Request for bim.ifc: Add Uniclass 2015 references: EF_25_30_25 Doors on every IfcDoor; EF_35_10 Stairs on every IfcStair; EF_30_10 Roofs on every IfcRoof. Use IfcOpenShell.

First a look at what the model holds.

```python
import ifcopenshell

model = ifcopenshell.open("bim.ifc")
print(model.schema)
print("classifications:", [c.Name for c in model.by_type("IfcClassification")])
for ifc_class in ("IfcDoor", "IfcRoof", "IfcStair", "IfcWall", "IfcWindow"):
    print(ifc_class, len(model.by_type(ifc_class)))
```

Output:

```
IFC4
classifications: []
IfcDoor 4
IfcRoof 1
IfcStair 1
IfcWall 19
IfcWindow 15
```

```python
import ifcopenshell
import ifcopenshell.api.classification

model = ifcopenshell.open("bim.ifc")

system = ifcopenshell.api.classification.add_classification(model, classification="Uniclass 2015")

codes = {
    "IfcDoor": ("EF_25_30_25", "Doors"),
    "IfcStair": ("EF_35_10", "Stairs"),
    "IfcRoof": ("EF_30_10", "Roofs"),
}
for ifc_class, (code, name) in codes.items():
    products = model.by_type(ifc_class)
    ifcopenshell.api.classification.add_reference(
        model, products=products, classification=system, identification=code, name=name
    )
    print(code, len(products))

model.write("bim_rev.ifc")
```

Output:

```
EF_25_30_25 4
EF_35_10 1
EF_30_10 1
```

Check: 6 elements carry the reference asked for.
